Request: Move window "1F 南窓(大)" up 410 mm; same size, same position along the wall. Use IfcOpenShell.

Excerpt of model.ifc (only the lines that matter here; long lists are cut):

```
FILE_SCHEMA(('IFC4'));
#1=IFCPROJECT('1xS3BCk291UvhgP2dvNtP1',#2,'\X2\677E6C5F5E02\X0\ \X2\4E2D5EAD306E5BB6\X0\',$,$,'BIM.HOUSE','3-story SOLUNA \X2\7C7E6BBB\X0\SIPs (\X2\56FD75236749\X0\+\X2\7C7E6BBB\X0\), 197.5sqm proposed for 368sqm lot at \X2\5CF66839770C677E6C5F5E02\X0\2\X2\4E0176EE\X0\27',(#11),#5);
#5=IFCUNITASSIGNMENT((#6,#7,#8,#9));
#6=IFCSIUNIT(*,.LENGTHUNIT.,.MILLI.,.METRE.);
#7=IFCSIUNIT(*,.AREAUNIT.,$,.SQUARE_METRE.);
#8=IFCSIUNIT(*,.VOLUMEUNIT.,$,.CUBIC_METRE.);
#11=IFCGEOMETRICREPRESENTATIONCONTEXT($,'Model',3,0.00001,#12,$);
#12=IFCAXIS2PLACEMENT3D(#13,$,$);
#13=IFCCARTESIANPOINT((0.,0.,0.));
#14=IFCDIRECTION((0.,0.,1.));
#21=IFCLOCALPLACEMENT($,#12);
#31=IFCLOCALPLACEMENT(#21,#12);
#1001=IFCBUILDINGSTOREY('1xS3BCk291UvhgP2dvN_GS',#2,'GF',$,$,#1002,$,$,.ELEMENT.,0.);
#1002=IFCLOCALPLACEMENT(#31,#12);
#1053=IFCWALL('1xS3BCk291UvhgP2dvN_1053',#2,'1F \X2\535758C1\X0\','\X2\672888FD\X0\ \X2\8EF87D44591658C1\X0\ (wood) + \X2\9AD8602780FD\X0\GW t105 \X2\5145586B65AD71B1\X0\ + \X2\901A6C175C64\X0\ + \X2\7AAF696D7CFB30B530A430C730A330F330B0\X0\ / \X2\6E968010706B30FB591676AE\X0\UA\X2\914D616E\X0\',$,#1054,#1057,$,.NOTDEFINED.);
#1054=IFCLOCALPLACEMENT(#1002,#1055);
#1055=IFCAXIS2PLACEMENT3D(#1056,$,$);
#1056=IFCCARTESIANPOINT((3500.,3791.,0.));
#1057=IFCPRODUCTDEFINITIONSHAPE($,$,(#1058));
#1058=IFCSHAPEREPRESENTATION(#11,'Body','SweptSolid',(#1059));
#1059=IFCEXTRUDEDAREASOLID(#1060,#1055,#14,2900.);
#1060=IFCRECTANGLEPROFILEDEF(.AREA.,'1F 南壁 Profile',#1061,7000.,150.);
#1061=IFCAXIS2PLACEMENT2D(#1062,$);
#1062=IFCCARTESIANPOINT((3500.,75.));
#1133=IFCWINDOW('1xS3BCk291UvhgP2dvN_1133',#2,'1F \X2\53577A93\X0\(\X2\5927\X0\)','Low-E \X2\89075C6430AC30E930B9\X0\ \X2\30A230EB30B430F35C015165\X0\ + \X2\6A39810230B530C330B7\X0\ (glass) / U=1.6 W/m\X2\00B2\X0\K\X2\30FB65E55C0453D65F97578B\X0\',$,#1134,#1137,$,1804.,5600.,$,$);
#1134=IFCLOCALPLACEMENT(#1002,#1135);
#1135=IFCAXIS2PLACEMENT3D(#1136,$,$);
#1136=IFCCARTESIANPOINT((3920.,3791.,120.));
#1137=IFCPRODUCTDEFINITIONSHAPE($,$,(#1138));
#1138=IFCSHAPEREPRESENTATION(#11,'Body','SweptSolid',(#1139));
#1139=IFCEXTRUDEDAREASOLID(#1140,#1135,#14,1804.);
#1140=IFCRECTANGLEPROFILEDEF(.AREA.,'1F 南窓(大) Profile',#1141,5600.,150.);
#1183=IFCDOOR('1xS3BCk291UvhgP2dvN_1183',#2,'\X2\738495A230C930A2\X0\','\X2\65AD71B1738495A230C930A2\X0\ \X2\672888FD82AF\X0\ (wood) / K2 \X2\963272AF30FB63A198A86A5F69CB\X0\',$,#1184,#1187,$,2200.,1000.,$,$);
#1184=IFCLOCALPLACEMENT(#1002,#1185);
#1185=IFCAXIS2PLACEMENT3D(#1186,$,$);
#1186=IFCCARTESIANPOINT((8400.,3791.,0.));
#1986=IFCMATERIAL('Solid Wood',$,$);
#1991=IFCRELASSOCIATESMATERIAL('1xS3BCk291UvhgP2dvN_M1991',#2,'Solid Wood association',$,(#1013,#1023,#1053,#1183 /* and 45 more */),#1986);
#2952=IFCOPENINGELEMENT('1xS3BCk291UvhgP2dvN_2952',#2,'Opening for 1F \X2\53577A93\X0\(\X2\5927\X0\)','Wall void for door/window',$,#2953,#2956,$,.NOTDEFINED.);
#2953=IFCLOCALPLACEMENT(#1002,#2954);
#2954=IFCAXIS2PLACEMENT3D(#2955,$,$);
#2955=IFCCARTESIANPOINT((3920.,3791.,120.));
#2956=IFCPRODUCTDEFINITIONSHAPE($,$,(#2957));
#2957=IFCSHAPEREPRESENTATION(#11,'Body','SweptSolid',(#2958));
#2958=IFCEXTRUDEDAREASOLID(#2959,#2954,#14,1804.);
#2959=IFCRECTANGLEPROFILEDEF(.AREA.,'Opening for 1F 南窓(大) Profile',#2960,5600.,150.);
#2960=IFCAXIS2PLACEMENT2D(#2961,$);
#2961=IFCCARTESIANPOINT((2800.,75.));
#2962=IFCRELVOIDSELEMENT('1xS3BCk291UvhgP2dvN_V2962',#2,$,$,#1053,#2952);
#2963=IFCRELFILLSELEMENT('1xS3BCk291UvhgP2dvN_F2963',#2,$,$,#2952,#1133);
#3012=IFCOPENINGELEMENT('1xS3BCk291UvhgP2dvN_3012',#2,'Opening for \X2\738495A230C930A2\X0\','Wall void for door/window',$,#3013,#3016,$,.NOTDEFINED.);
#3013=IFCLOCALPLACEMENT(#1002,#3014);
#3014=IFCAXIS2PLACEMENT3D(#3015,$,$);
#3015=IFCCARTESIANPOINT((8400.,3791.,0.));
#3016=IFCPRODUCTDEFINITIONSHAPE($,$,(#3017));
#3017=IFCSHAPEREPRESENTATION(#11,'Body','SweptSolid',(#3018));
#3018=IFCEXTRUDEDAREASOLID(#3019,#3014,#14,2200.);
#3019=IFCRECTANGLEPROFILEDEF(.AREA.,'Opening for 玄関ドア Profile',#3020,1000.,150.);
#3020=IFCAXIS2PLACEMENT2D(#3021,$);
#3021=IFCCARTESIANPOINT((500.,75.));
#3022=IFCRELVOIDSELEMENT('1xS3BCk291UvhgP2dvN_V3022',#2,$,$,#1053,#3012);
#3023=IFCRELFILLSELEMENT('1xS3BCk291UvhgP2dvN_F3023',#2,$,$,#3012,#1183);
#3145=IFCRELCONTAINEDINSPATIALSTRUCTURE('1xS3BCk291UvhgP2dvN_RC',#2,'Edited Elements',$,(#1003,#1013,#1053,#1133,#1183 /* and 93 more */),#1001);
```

```python
import numpy as np
import ifcopenshell
import ifcopenshell.api.geometry
import ifcopenshell.util.placement
import ifcopenshell.util.unit

model = ifcopenshell.open("model.ifc")
unit_scale = ifcopenshell.util.unit.calculate_unit_scale(model)

window = model.by_id(1133)
opening = window.FillsVoids[0].RelatingOpeningElement
dz = 0.41 / unit_scale

shift = np.array([0.0, 0.0, dz])
# The window is not placed relative to its opening, so move both.
for product in (opening, window):
    matrix = ifcopenshell.util.placement.get_local_placement(product.ObjectPlacement)
    matrix[:3, 3] += shift
    ifcopenshell.api.geometry.edit_object_placement(model, product=product, matrix=matrix, is_si=False)

print(f"moved by {dz * unit_scale:+.3f} m")

model.write("model_edited.ifc")
```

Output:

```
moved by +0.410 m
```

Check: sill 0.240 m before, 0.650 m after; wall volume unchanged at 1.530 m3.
